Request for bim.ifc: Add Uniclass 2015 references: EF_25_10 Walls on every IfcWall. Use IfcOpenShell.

First a look at what the model holds.

```python
import ifcopenshell

model = ifcopenshell.open("bim.ifc")
print(model.schema)
print("classifications:", [c.Name for c in model.by_type("IfcClassification")])
for ifc_class in ("IfcDoor", "IfcRoof", "IfcStair", "IfcWall", "IfcWindow"):
    print(ifc_class, len(model.by_type(ifc_class)))
```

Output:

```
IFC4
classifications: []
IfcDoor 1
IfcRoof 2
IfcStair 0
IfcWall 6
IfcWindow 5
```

```python
import ifcopenshell
import ifcopenshell.api.classification

model = ifcopenshell.open("bim.ifc")

system = ifcopenshell.api.classification.add_classification(model, classification="Uniclass 2015")

codes = {
    "IfcWall": ("EF_25_10", "Walls"),
}
for ifc_class, (code, name) in codes.items():
    products = model.by_type(ifc_class)
    ifcopenshell.api.classification.add_reference(
        model, products=products, classification=system, identification=code, name=name
    )
    print(code, len(products))

model.write("bim_updated.ifc")
```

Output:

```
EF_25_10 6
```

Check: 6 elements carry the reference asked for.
